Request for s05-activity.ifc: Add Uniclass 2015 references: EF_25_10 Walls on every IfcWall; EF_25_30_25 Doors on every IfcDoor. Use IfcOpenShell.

First a look at what the model holds.

```python
import ifcopenshell

model = ifcopenshell.open("s05-activity.ifc")
print(model.schema)
print("classifications:", [c.Name for c in model.by_type("IfcClassification")])
for ifc_class in ("IfcDoor", "IfcRoof", "IfcStair", "IfcWall", "IfcWindow"):
    print(ifc_class, len(model.by_type(ifc_class)))
```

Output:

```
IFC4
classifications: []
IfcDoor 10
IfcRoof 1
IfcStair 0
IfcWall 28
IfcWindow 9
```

```python
import ifcopenshell
import ifcopenshell.api.classification

model = ifcopenshell.open("s05-activity.ifc")

system = ifcopenshell.api.classification.add_classification(model, classification="Uniclass 2015")

codes = {
    "IfcWall": ("EF_25_10", "Walls"),
    "IfcDoor": ("EF_25_30_25", "Doors"),
}
for ifc_class, (code, name) in codes.items():
    products = model.by_type(ifc_class)
    ifcopenshell.api.classification.add_reference(
        model, products=products, classification=system, identification=code, name=name
    )
    print(code, len(products))

model.write("s05-activity_v2.ifc")
```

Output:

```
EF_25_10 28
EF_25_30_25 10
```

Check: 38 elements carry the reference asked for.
